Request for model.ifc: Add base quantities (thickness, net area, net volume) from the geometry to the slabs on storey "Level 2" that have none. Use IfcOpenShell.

First a look at what the model holds.

```python
import ifcopenshell
import ifcopenshell.util.element
import ifcopenshell.util.unit

model = ifcopenshell.open("model.ifc")
print(model.schema)
for unit_type in ("LENGTHUNIT", "AREAUNIT", "VOLUMEUNIT"):
    print(unit_type, ifcopenshell.util.unit.calculate_unit_scale(model, unit_type))
storey = next(s for s in model.by_type("IfcBuildingStorey") if s.Name == "Level 2")
slabs = [e for e in ifcopenshell.util.element.get_decomposition(storey) if e.is_a("IfcSlab")]
for e in sorted(slabs, key=lambda e: e.id()):
    print(e.id(), e.is_a(), e.Name, list(ifcopenshell.util.element.get_psets(e, qtos_only=True)), sep=" | ")
```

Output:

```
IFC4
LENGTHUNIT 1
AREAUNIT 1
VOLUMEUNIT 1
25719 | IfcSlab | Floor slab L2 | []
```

```python
import ifcopenshell
import ifcopenshell.api.pset
import ifcopenshell.geom
import ifcopenshell.util.element
import ifcopenshell.util.shape
import ifcopenshell.util.unit

model = ifcopenshell.open("model.ifc")
unit_scale = ifcopenshell.util.unit.calculate_unit_scale(model)
area_scale = ifcopenshell.util.unit.calculate_unit_scale(model, "AREAUNIT")
volume_scale = ifcopenshell.util.unit.calculate_unit_scale(model, "VOLUMEUNIT")
settings = ifcopenshell.geom.settings()

storey = next(s for s in model.by_type("IfcBuildingStorey") if s.Name == "Level 2")
slabs = [e for e in ifcopenshell.util.element.get_decomposition(storey) if e.is_a("IfcSlab")]

for e in sorted(slabs, key=lambda e: e.id()):
    if ifcopenshell.util.element.get_psets(e, qtos_only=True, should_inherit=False):
        continue
    # Geometry comes back in metres, in the element's own axes.
    shape = ifcopenshell.geom.create_shape(settings, e)
    values = {
        "Width": ifcopenshell.util.shape.get_z(shape.geometry) / unit_scale,
        "NetArea": ifcopenshell.util.shape.get_footprint_area(shape.geometry) / area_scale,
        "NetVolume": ifcopenshell.util.shape.get_volume(shape.geometry) / volume_scale,
    }
    qto = ifcopenshell.api.pset.add_qto(model, product=e, name="Qto_SlabBaseQuantities")
    ifcopenshell.api.pset.edit_qto(model, qto=qto, properties=values)
    print(e.id(), {k: round(v, 3) for k, v in values.items()})

model.write("model_v2.ifc")
```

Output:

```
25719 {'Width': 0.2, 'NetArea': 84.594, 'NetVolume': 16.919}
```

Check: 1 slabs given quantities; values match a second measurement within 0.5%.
